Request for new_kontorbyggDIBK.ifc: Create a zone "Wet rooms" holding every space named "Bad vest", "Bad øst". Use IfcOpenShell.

First a look at what the model holds.

```python
import ifcopenshell

model = ifcopenshell.open("new_kontorbyggDIBK.ifc")
print(model.schema)
seen = {}
for space in model.by_type("IfcSpace"):
    seen[space.LongName] = seen.get(space.LongName, 0) + 1
for name, count in sorted(seen.items(), key=str):
    print(count, "x", name)
print("zones:", [z.Name for z in model.by_type("IfcZone")][:20])
```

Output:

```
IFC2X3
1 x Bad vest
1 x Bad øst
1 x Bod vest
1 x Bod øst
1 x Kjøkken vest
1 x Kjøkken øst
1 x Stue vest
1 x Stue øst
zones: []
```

```python
import ifcopenshell
import ifcopenshell.api.group
import ifcopenshell.api.root

model = ifcopenshell.open("new_kontorbyggDIBK.ifc")

names = {"Bad vest", "Bad øst"}
spaces = [s for s in model.by_type("IfcSpace") if s.LongName in names]

zone = ifcopenshell.api.root.create_entity(model, ifc_class="IfcZone", name="Wet rooms")
ifcopenshell.api.group.assign_group(model, products=spaces, group=zone)
print(len(spaces), "spaces in", zone.Name)

model.write("new_kontorbyggDIBK_v2.ifc")
```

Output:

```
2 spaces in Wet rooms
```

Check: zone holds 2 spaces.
